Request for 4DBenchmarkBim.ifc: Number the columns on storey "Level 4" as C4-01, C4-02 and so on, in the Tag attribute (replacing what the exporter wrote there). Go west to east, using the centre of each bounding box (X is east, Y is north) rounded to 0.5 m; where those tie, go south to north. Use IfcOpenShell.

First a look at what the model holds.

```python
import ifcopenshell
import ifcopenshell.util.element
import ifcopenshell.util.placement

model = ifcopenshell.open("4DBenchmarkBim.ifc")
print(model.schema)
storey = next(s for s in model.by_type("IfcBuildingStorey") if s.Name == "Level 4")
columns = [e for e in ifcopenshell.util.element.get_decomposition(storey) if e.is_a("IfcColumn")]
for e in sorted(columns, key=lambda e: e.id()):
    origin = ifcopenshell.util.placement.get_local_placement(e.ObjectPlacement)[:3, 3]
    print(e.id(), e.Tag, e.Name, origin.round(2) + 0.0, sep=" | ")
```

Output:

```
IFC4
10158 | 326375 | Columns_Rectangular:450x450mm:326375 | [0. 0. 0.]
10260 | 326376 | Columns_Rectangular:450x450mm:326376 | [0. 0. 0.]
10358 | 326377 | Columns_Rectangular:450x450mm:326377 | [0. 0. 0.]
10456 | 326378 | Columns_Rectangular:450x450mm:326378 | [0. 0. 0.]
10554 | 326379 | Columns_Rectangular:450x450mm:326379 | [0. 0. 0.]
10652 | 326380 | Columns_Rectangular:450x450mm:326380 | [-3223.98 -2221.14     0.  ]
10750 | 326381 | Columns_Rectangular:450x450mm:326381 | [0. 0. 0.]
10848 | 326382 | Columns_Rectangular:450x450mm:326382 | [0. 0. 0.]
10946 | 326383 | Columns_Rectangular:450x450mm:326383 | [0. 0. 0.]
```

```python
import ifcopenshell
import ifcopenshell.geom
import ifcopenshell.util.element
import ifcopenshell.util.shape

model = ifcopenshell.open("4DBenchmarkBim.ifc")
settings = ifcopenshell.geom.settings()
settings.set("use-world-coords", True)


def centre(element):
    shape = ifcopenshell.geom.create_shape(settings, element)
    return ifcopenshell.util.shape.get_bbox_centroid(shape.geometry)


storey = next(s for s in model.by_type("IfcBuildingStorey") if s.Name == "Level 4")
columns = [e for e in ifcopenshell.util.element.get_decomposition(storey) if e.is_a("IfcColumn")]

# Insertion points can sit at a corner or the storey origin, so sort by the geometry (in metres).
centres = {e: centre(e) for e in columns}
columns.sort(key=lambda e: (round(centres[e][0] / 0.5), centres[e][1]))

for i, e in enumerate(columns, start=1):
    number = f"C4-{i:02d}"
    e.Tag = number
    print(e.id(), number)

model.write("4DBenchmarkBim_updated.ifc")
```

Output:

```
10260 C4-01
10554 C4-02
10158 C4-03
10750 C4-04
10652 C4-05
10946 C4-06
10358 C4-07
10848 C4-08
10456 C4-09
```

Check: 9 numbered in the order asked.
